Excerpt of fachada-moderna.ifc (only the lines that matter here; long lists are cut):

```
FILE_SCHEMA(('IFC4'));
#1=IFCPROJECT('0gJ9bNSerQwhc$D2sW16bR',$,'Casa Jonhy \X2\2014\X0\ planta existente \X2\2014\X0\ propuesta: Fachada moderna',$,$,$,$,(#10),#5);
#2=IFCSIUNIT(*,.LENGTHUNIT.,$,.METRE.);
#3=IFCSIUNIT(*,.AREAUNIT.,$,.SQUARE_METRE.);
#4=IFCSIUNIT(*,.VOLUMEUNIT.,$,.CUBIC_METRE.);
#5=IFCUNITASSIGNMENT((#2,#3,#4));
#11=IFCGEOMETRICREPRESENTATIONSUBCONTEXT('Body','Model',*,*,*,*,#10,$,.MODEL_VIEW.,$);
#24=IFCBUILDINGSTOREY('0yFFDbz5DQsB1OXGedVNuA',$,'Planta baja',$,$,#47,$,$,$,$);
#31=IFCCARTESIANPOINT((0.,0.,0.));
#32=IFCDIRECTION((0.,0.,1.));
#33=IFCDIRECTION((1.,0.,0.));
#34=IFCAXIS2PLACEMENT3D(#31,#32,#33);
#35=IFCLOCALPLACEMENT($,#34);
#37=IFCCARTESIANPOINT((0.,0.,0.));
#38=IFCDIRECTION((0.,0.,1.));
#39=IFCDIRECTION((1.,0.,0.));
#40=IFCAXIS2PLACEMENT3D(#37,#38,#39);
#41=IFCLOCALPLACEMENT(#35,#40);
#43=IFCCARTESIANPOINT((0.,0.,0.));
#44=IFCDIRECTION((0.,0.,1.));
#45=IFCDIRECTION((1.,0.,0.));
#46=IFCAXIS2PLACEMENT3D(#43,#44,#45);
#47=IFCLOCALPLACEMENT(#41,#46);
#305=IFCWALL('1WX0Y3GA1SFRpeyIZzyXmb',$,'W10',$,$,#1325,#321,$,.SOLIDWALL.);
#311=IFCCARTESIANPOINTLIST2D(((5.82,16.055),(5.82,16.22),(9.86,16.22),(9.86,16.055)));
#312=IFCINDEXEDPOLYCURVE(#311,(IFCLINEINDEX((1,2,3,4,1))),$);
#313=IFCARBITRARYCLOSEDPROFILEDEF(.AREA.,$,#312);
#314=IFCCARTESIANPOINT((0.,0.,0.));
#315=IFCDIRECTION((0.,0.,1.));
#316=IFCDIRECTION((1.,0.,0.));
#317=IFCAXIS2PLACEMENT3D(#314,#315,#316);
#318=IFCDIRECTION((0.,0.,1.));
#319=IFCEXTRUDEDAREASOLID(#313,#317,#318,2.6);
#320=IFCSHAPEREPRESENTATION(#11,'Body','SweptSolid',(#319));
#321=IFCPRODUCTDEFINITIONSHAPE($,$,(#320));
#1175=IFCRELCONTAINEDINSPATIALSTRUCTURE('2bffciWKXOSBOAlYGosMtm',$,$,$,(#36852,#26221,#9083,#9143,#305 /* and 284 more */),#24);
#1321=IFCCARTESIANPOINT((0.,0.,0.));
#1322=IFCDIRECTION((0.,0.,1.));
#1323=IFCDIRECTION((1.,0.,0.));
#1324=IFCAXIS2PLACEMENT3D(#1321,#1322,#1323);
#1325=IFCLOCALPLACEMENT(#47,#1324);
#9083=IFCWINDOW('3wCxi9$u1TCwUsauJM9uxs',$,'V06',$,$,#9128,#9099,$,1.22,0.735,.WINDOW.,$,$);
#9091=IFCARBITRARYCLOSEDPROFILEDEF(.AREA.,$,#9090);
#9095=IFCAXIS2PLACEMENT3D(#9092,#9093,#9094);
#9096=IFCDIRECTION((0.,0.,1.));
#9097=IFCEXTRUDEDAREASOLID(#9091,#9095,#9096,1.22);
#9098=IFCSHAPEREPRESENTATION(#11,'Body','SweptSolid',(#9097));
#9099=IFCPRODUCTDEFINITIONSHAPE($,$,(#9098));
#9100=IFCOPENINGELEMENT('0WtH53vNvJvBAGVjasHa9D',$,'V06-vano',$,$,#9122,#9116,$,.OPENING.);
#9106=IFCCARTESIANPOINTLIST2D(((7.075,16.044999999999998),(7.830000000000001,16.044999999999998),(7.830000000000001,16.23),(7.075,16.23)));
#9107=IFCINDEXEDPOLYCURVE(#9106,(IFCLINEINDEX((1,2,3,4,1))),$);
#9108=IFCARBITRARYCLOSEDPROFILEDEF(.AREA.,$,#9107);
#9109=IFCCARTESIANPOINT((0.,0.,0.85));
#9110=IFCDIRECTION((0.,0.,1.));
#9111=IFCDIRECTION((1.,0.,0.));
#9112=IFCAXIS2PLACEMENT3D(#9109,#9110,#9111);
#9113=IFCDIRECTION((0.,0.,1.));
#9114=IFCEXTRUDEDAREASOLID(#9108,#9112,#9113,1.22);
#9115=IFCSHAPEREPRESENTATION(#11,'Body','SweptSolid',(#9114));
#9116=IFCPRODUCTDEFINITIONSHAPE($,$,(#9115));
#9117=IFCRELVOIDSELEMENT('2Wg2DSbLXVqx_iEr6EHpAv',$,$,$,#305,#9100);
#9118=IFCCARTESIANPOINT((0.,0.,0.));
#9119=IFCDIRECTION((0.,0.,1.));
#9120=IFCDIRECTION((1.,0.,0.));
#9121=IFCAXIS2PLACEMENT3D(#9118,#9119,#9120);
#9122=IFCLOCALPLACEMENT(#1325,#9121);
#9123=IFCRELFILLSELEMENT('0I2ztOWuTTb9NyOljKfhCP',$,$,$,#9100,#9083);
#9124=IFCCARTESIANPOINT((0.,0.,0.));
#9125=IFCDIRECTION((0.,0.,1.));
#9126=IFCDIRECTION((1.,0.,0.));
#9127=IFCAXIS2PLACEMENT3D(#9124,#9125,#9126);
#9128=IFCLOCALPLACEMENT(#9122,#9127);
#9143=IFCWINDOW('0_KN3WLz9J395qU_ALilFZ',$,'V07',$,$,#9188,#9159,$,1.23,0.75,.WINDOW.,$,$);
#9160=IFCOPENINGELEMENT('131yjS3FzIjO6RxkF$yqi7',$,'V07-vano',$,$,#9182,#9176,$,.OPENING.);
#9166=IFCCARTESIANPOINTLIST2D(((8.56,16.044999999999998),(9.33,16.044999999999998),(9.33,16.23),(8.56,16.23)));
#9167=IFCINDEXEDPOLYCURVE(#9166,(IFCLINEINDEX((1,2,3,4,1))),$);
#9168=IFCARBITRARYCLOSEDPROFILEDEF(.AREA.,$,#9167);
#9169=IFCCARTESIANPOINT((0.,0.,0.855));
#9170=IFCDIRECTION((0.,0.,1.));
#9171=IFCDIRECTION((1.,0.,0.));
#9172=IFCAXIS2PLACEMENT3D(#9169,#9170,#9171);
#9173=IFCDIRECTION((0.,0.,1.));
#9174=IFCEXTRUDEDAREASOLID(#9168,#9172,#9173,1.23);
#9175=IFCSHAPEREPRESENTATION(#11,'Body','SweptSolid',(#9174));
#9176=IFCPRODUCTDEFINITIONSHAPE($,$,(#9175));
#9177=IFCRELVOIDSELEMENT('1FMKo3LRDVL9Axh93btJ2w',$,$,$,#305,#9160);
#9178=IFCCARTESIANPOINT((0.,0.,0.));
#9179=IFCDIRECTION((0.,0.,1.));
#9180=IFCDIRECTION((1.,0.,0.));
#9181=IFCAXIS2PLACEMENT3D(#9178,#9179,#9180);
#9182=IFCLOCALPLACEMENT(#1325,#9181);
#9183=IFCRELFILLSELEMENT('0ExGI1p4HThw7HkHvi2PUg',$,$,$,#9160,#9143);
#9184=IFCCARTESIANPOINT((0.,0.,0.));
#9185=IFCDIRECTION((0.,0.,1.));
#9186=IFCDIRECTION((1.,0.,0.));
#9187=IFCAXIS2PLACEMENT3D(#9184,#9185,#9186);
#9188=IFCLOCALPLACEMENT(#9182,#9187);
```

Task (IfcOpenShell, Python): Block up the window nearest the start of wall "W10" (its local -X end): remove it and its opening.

```python
import ifcopenshell
import ifcopenshell.api.feature
import ifcopenshell.api.root
import ifcopenshell.geom
import ifcopenshell.util.shape

model = ifcopenshell.open("fachada-moderna.ifc")
settings = ifcopenshell.geom.settings()


def volume(element):
    """Net volume in cubic metres, openings subtracted."""
    shape = ifcopenshell.geom.create_shape(settings, element)
    return ifcopenshell.util.shape.get_volume(shape.geometry)


window = model.by_id(9083)
opening = window.FillsVoids[0].RelatingOpeningElement
wall = opening.VoidsElements[0].RelatingBuildingElement
before = volume(wall)

ifcopenshell.api.root.remove_product(model, product=window)
ifcopenshell.api.feature.remove_feature(model, feature=opening)

after = volume(wall)

print(f"wall volume {before:.3f} -> {after:.3f} m3")

model.write("fachada-moderna_edited.ifc")
```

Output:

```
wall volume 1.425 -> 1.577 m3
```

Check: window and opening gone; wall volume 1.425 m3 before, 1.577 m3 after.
